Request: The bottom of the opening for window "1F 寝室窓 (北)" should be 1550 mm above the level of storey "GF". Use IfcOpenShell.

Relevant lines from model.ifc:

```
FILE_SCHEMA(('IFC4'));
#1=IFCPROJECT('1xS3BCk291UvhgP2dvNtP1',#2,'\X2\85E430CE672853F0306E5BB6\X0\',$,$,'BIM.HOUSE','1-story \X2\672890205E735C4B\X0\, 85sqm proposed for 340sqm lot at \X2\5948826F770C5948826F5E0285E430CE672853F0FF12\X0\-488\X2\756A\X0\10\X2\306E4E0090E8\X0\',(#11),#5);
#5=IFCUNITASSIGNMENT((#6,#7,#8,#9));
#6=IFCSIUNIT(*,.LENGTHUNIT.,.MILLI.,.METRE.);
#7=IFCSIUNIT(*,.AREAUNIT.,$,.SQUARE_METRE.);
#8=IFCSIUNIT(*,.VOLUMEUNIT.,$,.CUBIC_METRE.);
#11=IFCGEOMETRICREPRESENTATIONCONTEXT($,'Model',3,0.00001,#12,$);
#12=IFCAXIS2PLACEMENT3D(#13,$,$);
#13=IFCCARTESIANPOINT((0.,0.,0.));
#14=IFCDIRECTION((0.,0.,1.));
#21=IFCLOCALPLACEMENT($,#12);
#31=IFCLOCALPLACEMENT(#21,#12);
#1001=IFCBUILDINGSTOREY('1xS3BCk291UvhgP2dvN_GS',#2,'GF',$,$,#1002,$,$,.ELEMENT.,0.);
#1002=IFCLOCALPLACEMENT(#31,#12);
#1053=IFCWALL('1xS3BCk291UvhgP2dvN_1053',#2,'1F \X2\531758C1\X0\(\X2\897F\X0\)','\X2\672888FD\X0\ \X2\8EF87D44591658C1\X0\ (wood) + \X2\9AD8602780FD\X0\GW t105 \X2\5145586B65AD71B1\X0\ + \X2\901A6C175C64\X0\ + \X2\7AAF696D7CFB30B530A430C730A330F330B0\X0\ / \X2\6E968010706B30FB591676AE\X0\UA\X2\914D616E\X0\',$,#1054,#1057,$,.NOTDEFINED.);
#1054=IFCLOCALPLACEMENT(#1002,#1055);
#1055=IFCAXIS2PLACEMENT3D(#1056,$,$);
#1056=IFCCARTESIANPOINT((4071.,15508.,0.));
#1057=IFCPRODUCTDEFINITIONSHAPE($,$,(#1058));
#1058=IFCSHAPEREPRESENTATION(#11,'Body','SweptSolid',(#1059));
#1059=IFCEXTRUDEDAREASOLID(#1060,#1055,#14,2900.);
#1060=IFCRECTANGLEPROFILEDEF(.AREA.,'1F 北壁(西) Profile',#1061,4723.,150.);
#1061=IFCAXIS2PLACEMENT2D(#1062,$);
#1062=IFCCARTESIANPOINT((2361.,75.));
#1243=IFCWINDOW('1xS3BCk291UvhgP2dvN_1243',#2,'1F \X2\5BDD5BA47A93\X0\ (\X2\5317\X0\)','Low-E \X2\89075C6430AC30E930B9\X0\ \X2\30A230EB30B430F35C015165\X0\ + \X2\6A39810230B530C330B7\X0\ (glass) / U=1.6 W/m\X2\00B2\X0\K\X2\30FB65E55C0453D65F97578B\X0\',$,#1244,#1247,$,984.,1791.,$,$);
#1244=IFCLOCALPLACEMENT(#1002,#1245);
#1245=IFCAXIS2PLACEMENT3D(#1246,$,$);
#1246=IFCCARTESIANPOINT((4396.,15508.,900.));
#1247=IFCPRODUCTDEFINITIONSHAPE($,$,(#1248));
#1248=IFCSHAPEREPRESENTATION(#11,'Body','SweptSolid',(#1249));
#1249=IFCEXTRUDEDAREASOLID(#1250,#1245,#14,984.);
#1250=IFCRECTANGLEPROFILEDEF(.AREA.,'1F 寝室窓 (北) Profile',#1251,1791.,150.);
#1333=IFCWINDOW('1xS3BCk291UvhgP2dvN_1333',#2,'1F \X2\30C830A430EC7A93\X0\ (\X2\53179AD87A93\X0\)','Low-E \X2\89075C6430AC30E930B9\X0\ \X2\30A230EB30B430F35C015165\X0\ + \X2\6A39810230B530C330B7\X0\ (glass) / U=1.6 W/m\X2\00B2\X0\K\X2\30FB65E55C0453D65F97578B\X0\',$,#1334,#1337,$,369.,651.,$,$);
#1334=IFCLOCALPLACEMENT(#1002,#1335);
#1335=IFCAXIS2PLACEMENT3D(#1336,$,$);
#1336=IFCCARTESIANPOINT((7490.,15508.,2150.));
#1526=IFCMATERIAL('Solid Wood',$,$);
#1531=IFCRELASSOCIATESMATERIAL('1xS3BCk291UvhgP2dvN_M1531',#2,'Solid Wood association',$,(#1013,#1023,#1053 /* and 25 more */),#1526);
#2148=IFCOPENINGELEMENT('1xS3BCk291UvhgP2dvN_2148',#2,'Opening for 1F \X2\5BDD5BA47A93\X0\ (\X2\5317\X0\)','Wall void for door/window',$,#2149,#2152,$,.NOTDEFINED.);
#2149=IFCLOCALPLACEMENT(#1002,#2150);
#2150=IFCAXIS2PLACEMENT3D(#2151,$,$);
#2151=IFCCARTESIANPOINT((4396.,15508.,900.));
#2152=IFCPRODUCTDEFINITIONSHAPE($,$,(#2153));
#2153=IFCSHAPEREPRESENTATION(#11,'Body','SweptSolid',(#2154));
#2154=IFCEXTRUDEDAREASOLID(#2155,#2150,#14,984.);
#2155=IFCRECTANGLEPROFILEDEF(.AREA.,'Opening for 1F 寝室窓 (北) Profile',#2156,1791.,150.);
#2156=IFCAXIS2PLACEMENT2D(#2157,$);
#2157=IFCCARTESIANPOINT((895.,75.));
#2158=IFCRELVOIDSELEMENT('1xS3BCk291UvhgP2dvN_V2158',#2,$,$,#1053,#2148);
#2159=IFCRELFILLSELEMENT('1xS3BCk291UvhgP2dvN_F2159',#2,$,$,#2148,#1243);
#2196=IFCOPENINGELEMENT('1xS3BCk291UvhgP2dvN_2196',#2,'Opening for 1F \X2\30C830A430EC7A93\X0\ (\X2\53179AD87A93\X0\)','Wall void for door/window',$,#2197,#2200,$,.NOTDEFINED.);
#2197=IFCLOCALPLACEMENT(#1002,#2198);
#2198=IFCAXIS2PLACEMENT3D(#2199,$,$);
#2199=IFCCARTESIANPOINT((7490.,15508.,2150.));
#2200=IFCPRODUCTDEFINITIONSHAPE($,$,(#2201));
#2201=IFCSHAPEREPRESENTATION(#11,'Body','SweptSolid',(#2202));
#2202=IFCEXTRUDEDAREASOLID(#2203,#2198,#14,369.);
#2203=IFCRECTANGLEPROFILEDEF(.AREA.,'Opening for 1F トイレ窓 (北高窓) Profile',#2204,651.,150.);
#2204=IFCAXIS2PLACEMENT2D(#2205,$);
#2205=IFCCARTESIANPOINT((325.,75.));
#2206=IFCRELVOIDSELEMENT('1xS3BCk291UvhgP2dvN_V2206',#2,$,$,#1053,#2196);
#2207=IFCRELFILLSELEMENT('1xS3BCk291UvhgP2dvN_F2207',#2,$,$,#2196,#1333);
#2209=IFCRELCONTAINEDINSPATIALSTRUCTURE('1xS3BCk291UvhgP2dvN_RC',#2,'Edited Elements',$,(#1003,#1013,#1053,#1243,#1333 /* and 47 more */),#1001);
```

```python
import numpy as np
import ifcopenshell
import ifcopenshell.api.geometry
import ifcopenshell.geom
import ifcopenshell.util.element
import ifcopenshell.util.placement
import ifcopenshell.util.shape
import ifcopenshell.util.unit

model = ifcopenshell.open("model.ifc")
unit_scale = ifcopenshell.util.unit.calculate_unit_scale(model)

window = model.by_guid("1xS3BCk291UvhgP2dvN_1243")
opening = window.FillsVoids[0].RelatingOpeningElement
storey = ifcopenshell.util.element.get_container(window, ifc_class="IfcBuildingStorey")
level = ifcopenshell.util.placement.get_local_placement(storey.ObjectPlacement)[2, 3]

# The opening's origin need not be at the sill, so measure its lowest point.
shape = ifcopenshell.geom.create_shape(ifcopenshell.geom.settings(), opening)
bottom = ifcopenshell.util.shape.get_shape_bottom_elevation(shape, shape.geometry) / unit_scale
dz = level + 1.55 / unit_scale - bottom

shift = np.array([0.0, 0.0, dz])
# The window is not placed relative to its opening, so move both.
for product in (opening, window):
    matrix = ifcopenshell.util.placement.get_local_placement(product.ObjectPlacement)
    matrix[:3, 3] += shift
    ifcopenshell.api.geometry.edit_object_placement(model, product=product, matrix=matrix, is_si=False)

print(f"moved by {dz * unit_scale:+.3f} m")

model.write("model-out.ifc")
```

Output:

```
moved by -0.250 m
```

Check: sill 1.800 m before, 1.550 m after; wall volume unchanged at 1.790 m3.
